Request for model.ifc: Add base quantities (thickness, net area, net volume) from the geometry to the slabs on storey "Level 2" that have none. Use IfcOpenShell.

First a look at what the model holds.

```python
import ifcopenshell
import ifcopenshell.util.element
import ifcopenshell.util.unit

model = ifcopenshell.open("model.ifc")
print(model.schema)
for unit_type in ("LENGTHUNIT", "AREAUNIT", "VOLUMEUNIT"):
    print(unit_type, ifcopenshell.util.unit.calculate_unit_scale(model, unit_type))
storey = next(s for s in model.by_type("IfcBuildingStorey") if s.Name == "Level 2")
slabs = [e for e in ifcopenshell.util.element.get_decomposition(storey) if e.is_a("IfcSlab")]
for e in sorted(slabs, key=lambda e: e.id()):
    print(e.id(), e.is_a(), e.Name, list(ifcopenshell.util.element.get_psets(e, qtos_only=True)), sep=" | ")
```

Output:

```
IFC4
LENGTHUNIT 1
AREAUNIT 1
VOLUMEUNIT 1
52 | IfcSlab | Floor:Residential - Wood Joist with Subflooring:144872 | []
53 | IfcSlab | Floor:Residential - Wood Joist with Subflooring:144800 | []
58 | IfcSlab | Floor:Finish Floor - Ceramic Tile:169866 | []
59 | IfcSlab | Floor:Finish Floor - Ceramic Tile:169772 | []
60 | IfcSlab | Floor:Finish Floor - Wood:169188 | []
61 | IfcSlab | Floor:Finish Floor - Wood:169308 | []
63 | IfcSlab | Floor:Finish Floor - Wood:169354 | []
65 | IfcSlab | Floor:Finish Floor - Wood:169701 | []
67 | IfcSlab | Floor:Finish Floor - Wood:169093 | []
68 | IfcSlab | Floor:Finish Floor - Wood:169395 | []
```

```python
import ifcopenshell
import ifcopenshell.api.pset
import ifcopenshell.geom
import ifcopenshell.util.element
import ifcopenshell.util.shape
import ifcopenshell.util.unit

model = ifcopenshell.open("model.ifc")
unit_scale = ifcopenshell.util.unit.calculate_unit_scale(model)
area_scale = ifcopenshell.util.unit.calculate_unit_scale(model, "AREAUNIT")
volume_scale = ifcopenshell.util.unit.calculate_unit_scale(model, "VOLUMEUNIT")
settings = ifcopenshell.geom.settings()

storey = next(s for s in model.by_type("IfcBuildingStorey") if s.Name == "Level 2")
slabs = [e for e in ifcopenshell.util.element.get_decomposition(storey) if e.is_a("IfcSlab")]

for e in sorted(slabs, key=lambda e: e.id()):
    if ifcopenshell.util.element.get_psets(e, qtos_only=True, should_inherit=False):
        continue
    # Geometry comes back in metres, in the element's own axes.
    shape = ifcopenshell.geom.create_shape(settings, e)
    values = {
        "Width": ifcopenshell.util.shape.get_z(shape.geometry) / unit_scale,
        "NetArea": ifcopenshell.util.shape.get_footprint_area(shape.geometry) / area_scale,
        "NetVolume": ifcopenshell.util.shape.get_volume(shape.geometry) / volume_scale,
    }
    qto = ifcopenshell.api.pset.add_qto(model, product=e, name="Qto_SlabBaseQuantities")
    ifcopenshell.api.pset.edit_qto(model, qto=qto, properties=values)
    print(e.id(), {k: round(v, 3) for k, v in values.items()})

model.write("model_v2.ifc")
```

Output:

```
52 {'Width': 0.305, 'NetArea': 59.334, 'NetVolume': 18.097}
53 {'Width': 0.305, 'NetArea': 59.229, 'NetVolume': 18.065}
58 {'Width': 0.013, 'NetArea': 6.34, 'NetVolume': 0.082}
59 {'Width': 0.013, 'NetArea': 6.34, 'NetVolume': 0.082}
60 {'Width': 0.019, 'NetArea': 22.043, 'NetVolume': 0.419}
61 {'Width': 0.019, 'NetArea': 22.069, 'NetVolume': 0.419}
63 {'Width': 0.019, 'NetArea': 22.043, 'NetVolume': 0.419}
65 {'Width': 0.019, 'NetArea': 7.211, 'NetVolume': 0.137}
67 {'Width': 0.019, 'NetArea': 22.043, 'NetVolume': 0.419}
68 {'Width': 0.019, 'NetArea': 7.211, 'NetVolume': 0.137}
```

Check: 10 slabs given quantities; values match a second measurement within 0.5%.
